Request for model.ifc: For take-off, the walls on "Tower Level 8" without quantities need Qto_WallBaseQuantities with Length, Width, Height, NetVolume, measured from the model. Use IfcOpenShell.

First a look at what the model holds.

```python
import ifcopenshell
import ifcopenshell.util.element
import ifcopenshell.util.unit

model = ifcopenshell.open("model.ifc")
print(model.schema)
for unit_type in ("LENGTHUNIT", "AREAUNIT", "VOLUMEUNIT"):
    print(unit_type, ifcopenshell.util.unit.calculate_unit_scale(model, unit_type))
storey = next(s for s in model.by_type("IfcBuildingStorey") if s.Name == "Tower Level 8")
walls = [e for e in ifcopenshell.util.element.get_decomposition(storey) if e.is_a("IfcWall")]
for e in sorted(walls, key=lambda e: e.id()):
    print(e.id(), e.is_a(), e.Name, list(ifcopenshell.util.element.get_psets(e, qtos_only=True)), sep=" | ")
```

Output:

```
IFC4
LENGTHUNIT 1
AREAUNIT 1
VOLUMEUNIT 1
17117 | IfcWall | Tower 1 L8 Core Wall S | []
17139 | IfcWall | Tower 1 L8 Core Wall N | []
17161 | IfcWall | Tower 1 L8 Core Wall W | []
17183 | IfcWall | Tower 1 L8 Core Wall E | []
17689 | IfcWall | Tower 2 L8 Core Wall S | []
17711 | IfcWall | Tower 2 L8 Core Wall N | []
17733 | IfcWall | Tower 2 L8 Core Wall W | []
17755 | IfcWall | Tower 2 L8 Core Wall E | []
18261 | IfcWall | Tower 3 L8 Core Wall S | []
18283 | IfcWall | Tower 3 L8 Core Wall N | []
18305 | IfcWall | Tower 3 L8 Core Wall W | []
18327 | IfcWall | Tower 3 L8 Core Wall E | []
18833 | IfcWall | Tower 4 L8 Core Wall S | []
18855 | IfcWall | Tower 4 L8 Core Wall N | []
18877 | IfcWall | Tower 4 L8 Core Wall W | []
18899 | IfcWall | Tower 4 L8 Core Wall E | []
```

```python
import ifcopenshell
import ifcopenshell.api.pset
import ifcopenshell.geom
import ifcopenshell.util.element
import ifcopenshell.util.shape
import ifcopenshell.util.unit

model = ifcopenshell.open("model.ifc")
unit_scale = ifcopenshell.util.unit.calculate_unit_scale(model)
volume_scale = ifcopenshell.util.unit.calculate_unit_scale(model, "VOLUMEUNIT")
settings = ifcopenshell.geom.settings()

storey = next(s for s in model.by_type("IfcBuildingStorey") if s.Name == "Tower Level 8")
walls = [e for e in ifcopenshell.util.element.get_decomposition(storey) if e.is_a("IfcWall")]

for e in sorted(walls, key=lambda e: e.id()):
    if ifcopenshell.util.element.get_psets(e, qtos_only=True, should_inherit=False):
        continue
    # Geometry comes back in metres, in the element's own axes.
    shape = ifcopenshell.geom.create_shape(settings, e)
    values = {
        "Length": ifcopenshell.util.shape.get_x(shape.geometry) / unit_scale,
        "Width": ifcopenshell.util.shape.get_y(shape.geometry) / unit_scale,
        "Height": ifcopenshell.util.shape.get_z(shape.geometry) / unit_scale,
        "NetVolume": ifcopenshell.util.shape.get_volume(shape.geometry) / volume_scale,
    }
    qto = ifcopenshell.api.pset.add_qto(model, product=e, name="Qto_WallBaseQuantities")
    ifcopenshell.api.pset.edit_qto(model, qto=qto, properties=values)
    print(e.id(), {k: round(v, 3) for k, v in values.items()})

model.write("model_rev.ifc")
```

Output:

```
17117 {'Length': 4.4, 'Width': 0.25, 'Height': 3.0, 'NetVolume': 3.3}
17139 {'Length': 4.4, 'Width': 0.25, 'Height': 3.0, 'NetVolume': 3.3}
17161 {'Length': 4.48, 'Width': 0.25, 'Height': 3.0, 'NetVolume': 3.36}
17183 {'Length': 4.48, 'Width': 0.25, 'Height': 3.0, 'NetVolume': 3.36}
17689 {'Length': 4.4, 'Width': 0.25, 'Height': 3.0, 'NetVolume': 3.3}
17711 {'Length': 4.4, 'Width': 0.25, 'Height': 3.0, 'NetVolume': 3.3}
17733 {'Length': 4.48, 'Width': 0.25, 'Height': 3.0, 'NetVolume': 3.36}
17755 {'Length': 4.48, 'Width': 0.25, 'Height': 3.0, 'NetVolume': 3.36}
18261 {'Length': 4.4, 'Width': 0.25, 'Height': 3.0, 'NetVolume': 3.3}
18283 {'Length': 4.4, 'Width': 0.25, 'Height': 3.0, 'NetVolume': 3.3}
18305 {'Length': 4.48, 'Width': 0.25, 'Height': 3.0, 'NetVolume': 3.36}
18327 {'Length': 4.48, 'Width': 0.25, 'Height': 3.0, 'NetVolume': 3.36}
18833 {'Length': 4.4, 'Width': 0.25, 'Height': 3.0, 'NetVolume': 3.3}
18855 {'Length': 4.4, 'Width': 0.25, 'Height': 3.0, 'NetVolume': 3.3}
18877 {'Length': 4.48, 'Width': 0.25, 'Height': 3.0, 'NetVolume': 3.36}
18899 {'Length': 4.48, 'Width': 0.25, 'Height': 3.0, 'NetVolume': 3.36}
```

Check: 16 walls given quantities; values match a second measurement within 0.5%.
